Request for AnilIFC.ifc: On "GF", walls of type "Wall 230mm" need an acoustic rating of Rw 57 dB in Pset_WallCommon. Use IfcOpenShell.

First a look at what the model holds.

```python
import ifcopenshell
import ifcopenshell.util.element

model = ifcopenshell.open("AnilIFC.ifc")
print(model.schema)
storey = next(s for s in model.by_type("IfcBuildingStorey") if s.Name == "GF")
walls = [e for e in ifcopenshell.util.element.get_decomposition(storey) if e.is_a("IfcWall")]
seen = {}
for e in walls:
    element_type = ifcopenshell.util.element.get_type(e)
    key = (element_type.Name if element_type != e and element_type else None, ifcopenshell.util.element.get_pset(e, "Pset_WallCommon", "AcousticRating"))
    seen[key] = seen.get(key, 0) + 1
for (name, value), count in sorted(seen.items(), key=str):
    print(count, "x", name, "|", value)
```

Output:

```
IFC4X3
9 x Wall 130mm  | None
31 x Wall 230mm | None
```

```python
import ifcopenshell
import ifcopenshell.api.pset
import ifcopenshell.util.element

model = ifcopenshell.open("AnilIFC.ifc")

storey = next(s for s in model.by_type("IfcBuildingStorey") if s.Name == "GF")
walls = [e for e in ifcopenshell.util.element.get_decomposition(storey) if e.is_a("IfcWall")]

count = 0
for e in walls:
    element_type = ifcopenshell.util.element.get_type(e)
    if element_type in (None, e) or element_type.Name != "Wall 230mm":
        continue
    # add_pset returns the element's existing set when there is one.
    pset = ifcopenshell.api.pset.add_pset(model, product=e, name="Pset_WallCommon")
    ifcopenshell.api.pset.edit_pset(model, pset=pset, properties={"AcousticRating": "Rw 57 dB"})
    count += 1

print(count, "walls updated")

model.write("AnilIFC_edited.ifc")
```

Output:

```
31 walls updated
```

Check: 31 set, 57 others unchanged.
